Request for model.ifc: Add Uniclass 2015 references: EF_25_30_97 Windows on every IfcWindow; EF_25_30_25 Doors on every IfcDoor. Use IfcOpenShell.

First a look at what the model holds.

```python
import ifcopenshell

model = ifcopenshell.open("model.ifc")
print(model.schema)
print("classifications:", [c.Name for c in model.by_type("IfcClassification")])
for ifc_class in ("IfcDoor", "IfcRoof", "IfcStair", "IfcWall", "IfcWindow"):
    print(ifc_class, len(model.by_type(ifc_class)))
```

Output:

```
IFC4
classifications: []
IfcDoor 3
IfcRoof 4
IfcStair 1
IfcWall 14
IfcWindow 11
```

```python
import ifcopenshell
import ifcopenshell.api.classification

model = ifcopenshell.open("model.ifc")

system = ifcopenshell.api.classification.add_classification(model, classification="Uniclass 2015")

codes = {
    "IfcWindow": ("EF_25_30_97", "Windows"),
    "IfcDoor": ("EF_25_30_25", "Doors"),
}
for ifc_class, (code, name) in codes.items():
    products = model.by_type(ifc_class)
    ifcopenshell.api.classification.add_reference(
        model, products=products, classification=system, identification=code, name=name
    )
    print(code, len(products))

model.write("model_v2.ifc")
```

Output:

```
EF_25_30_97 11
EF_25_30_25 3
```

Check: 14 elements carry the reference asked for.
